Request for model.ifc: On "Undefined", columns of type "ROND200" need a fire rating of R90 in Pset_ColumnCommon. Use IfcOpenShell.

First a look at what the model holds.

```python
import ifcopenshell
import ifcopenshell.util.element

model = ifcopenshell.open("model.ifc")
print(model.schema)
storey = next(s for s in model.by_type("IfcBuildingStorey") if s.Name == "Undefined")
columns = [e for e in ifcopenshell.util.element.get_decomposition(storey) if e.is_a("IfcColumn")]
seen = {}
for e in columns:
    element_type = ifcopenshell.util.element.get_type(e)
    key = (element_type.Name if element_type != e and element_type else None, ifcopenshell.util.element.get_pset(e, "Pset_ColumnCommon", "FireRating"))
    seen[key] = seen.get(key, 0) + 1
for (name, value), count in sorted(seen.items(), key=str):
    print(count, "x", name, "|", value)
```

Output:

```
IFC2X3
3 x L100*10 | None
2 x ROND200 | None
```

```python
import ifcopenshell
import ifcopenshell.api.pset
import ifcopenshell.util.element

model = ifcopenshell.open("model.ifc")

storey = next(s for s in model.by_type("IfcBuildingStorey") if s.Name == "Undefined")
columns = [e for e in ifcopenshell.util.element.get_decomposition(storey) if e.is_a("IfcColumn")]

count = 0
for e in columns:
    element_type = ifcopenshell.util.element.get_type(e)
    if element_type in (None, e) or element_type.Name != "ROND200":
        continue
    # add_pset returns the element's existing set when there is one.
    pset = ifcopenshell.api.pset.add_pset(model, product=e, name="Pset_ColumnCommon")
    ifcopenshell.api.pset.edit_pset(model, pset=pset, properties={"FireRating": "R90"})
    count += 1

print(count, "columns updated")

model.write("model_edited.ifc")
```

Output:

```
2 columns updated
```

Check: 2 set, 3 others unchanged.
